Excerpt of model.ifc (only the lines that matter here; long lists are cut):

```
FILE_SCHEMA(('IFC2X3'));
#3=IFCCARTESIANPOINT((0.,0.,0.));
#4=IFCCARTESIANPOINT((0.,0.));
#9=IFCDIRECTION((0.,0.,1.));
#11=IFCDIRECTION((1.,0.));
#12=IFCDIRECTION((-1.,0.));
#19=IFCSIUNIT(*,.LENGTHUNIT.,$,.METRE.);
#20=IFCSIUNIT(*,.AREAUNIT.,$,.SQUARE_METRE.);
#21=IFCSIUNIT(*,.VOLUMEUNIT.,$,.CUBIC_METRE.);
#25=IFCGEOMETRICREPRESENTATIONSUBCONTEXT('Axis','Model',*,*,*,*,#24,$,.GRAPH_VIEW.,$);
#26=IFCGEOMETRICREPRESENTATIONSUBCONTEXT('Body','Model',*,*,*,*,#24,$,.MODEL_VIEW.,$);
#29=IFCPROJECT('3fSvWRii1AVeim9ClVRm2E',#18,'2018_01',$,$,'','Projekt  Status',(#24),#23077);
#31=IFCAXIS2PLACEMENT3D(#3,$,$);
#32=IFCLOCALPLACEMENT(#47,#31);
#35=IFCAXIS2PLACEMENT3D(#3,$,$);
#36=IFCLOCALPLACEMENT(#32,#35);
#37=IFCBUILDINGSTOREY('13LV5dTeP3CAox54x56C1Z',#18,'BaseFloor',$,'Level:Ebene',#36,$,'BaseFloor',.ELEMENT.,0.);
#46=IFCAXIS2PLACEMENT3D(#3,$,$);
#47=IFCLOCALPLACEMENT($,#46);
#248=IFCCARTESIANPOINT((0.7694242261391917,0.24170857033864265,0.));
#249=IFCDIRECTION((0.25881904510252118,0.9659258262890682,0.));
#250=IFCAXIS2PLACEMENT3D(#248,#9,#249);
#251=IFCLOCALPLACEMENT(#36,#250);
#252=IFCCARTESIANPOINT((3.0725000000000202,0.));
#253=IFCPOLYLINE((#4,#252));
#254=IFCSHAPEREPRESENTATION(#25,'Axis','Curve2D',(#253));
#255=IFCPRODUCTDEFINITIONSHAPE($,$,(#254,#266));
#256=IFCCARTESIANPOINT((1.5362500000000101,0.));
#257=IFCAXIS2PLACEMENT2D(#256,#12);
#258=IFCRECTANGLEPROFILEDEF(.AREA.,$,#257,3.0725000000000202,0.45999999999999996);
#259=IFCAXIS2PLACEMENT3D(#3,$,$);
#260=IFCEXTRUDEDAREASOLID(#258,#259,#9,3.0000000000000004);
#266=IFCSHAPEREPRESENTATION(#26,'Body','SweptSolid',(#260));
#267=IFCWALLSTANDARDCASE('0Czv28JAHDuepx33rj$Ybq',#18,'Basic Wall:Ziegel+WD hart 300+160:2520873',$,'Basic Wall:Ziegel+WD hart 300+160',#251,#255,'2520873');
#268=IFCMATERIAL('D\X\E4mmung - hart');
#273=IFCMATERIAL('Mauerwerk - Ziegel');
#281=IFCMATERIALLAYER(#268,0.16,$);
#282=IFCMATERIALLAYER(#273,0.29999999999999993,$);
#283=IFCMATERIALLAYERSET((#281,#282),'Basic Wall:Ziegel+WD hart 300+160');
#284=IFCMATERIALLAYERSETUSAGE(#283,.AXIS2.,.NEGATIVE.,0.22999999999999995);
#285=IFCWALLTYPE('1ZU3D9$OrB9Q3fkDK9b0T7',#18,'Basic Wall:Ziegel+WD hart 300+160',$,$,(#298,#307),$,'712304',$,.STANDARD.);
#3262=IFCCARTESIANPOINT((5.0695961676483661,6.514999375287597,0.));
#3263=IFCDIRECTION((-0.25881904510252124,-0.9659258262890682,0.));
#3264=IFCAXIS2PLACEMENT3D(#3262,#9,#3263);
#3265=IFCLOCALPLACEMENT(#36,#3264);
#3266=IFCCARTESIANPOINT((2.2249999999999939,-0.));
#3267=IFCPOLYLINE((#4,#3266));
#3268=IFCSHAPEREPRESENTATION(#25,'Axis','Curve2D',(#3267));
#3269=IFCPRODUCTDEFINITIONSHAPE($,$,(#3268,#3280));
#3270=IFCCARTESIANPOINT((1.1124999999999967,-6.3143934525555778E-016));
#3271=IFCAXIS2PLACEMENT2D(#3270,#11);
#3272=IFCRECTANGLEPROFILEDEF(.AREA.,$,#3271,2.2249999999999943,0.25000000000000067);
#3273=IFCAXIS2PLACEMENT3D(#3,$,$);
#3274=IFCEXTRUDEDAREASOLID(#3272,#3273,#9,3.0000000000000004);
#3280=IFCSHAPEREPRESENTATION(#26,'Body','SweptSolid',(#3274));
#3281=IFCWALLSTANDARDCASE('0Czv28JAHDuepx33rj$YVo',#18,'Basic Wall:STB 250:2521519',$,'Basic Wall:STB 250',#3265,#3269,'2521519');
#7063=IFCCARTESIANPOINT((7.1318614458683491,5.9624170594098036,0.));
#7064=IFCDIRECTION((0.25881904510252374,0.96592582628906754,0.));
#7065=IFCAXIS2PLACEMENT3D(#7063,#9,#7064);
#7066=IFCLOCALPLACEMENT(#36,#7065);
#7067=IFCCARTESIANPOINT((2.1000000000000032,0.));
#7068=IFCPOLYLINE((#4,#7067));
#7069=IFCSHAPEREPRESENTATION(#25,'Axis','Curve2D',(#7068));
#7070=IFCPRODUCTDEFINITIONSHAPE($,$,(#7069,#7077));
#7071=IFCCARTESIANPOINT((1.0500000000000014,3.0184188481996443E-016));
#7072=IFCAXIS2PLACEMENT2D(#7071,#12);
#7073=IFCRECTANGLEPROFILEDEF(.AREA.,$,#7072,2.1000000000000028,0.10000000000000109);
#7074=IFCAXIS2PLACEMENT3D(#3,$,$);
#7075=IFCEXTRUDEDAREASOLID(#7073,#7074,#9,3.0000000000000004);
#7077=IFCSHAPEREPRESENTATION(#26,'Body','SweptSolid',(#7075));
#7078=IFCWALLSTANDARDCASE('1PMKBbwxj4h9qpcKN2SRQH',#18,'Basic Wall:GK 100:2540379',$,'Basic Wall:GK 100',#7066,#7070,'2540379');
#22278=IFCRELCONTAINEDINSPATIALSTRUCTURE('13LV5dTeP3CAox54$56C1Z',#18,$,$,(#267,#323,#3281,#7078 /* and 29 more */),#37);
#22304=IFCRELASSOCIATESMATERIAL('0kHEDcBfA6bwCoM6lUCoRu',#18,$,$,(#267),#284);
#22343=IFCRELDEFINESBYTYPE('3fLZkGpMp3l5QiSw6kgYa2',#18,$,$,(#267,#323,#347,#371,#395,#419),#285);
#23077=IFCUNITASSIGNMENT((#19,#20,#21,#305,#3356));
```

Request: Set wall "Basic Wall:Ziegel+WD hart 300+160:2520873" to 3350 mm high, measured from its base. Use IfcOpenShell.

```python
import ifcopenshell
import ifcopenshell.geom
import ifcopenshell.util.representation
import ifcopenshell.util.shape
import ifcopenshell.util.unit

model = ifcopenshell.open("model.ifc")
unit_scale = ifcopenshell.util.unit.calculate_unit_scale(model)
settings = ifcopenshell.geom.settings()


def volume(element):
    """Net volume in cubic metres, openings subtracted."""
    shape = ifcopenshell.geom.create_shape(settings, element)
    return ifcopenshell.util.shape.get_volume(shape.geometry)


wall = model.by_guid("0Czv28JAHDuepx33rj$Ybq")
before = volume(wall)

body = ifcopenshell.util.representation.get_representation(wall, "Model", "Body")
solid = body.Items[0]
old_height = solid.Depth
solid.Depth = 3.35 / unit_scale
after = volume(wall)

print(f"height {old_height:g} -> {solid.Depth:g}, volume {before:.3f} -> {after:.3f} m3")

model.write("model_v2.ifc")
```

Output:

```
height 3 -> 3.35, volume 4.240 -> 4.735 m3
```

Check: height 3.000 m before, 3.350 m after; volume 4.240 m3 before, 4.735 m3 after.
